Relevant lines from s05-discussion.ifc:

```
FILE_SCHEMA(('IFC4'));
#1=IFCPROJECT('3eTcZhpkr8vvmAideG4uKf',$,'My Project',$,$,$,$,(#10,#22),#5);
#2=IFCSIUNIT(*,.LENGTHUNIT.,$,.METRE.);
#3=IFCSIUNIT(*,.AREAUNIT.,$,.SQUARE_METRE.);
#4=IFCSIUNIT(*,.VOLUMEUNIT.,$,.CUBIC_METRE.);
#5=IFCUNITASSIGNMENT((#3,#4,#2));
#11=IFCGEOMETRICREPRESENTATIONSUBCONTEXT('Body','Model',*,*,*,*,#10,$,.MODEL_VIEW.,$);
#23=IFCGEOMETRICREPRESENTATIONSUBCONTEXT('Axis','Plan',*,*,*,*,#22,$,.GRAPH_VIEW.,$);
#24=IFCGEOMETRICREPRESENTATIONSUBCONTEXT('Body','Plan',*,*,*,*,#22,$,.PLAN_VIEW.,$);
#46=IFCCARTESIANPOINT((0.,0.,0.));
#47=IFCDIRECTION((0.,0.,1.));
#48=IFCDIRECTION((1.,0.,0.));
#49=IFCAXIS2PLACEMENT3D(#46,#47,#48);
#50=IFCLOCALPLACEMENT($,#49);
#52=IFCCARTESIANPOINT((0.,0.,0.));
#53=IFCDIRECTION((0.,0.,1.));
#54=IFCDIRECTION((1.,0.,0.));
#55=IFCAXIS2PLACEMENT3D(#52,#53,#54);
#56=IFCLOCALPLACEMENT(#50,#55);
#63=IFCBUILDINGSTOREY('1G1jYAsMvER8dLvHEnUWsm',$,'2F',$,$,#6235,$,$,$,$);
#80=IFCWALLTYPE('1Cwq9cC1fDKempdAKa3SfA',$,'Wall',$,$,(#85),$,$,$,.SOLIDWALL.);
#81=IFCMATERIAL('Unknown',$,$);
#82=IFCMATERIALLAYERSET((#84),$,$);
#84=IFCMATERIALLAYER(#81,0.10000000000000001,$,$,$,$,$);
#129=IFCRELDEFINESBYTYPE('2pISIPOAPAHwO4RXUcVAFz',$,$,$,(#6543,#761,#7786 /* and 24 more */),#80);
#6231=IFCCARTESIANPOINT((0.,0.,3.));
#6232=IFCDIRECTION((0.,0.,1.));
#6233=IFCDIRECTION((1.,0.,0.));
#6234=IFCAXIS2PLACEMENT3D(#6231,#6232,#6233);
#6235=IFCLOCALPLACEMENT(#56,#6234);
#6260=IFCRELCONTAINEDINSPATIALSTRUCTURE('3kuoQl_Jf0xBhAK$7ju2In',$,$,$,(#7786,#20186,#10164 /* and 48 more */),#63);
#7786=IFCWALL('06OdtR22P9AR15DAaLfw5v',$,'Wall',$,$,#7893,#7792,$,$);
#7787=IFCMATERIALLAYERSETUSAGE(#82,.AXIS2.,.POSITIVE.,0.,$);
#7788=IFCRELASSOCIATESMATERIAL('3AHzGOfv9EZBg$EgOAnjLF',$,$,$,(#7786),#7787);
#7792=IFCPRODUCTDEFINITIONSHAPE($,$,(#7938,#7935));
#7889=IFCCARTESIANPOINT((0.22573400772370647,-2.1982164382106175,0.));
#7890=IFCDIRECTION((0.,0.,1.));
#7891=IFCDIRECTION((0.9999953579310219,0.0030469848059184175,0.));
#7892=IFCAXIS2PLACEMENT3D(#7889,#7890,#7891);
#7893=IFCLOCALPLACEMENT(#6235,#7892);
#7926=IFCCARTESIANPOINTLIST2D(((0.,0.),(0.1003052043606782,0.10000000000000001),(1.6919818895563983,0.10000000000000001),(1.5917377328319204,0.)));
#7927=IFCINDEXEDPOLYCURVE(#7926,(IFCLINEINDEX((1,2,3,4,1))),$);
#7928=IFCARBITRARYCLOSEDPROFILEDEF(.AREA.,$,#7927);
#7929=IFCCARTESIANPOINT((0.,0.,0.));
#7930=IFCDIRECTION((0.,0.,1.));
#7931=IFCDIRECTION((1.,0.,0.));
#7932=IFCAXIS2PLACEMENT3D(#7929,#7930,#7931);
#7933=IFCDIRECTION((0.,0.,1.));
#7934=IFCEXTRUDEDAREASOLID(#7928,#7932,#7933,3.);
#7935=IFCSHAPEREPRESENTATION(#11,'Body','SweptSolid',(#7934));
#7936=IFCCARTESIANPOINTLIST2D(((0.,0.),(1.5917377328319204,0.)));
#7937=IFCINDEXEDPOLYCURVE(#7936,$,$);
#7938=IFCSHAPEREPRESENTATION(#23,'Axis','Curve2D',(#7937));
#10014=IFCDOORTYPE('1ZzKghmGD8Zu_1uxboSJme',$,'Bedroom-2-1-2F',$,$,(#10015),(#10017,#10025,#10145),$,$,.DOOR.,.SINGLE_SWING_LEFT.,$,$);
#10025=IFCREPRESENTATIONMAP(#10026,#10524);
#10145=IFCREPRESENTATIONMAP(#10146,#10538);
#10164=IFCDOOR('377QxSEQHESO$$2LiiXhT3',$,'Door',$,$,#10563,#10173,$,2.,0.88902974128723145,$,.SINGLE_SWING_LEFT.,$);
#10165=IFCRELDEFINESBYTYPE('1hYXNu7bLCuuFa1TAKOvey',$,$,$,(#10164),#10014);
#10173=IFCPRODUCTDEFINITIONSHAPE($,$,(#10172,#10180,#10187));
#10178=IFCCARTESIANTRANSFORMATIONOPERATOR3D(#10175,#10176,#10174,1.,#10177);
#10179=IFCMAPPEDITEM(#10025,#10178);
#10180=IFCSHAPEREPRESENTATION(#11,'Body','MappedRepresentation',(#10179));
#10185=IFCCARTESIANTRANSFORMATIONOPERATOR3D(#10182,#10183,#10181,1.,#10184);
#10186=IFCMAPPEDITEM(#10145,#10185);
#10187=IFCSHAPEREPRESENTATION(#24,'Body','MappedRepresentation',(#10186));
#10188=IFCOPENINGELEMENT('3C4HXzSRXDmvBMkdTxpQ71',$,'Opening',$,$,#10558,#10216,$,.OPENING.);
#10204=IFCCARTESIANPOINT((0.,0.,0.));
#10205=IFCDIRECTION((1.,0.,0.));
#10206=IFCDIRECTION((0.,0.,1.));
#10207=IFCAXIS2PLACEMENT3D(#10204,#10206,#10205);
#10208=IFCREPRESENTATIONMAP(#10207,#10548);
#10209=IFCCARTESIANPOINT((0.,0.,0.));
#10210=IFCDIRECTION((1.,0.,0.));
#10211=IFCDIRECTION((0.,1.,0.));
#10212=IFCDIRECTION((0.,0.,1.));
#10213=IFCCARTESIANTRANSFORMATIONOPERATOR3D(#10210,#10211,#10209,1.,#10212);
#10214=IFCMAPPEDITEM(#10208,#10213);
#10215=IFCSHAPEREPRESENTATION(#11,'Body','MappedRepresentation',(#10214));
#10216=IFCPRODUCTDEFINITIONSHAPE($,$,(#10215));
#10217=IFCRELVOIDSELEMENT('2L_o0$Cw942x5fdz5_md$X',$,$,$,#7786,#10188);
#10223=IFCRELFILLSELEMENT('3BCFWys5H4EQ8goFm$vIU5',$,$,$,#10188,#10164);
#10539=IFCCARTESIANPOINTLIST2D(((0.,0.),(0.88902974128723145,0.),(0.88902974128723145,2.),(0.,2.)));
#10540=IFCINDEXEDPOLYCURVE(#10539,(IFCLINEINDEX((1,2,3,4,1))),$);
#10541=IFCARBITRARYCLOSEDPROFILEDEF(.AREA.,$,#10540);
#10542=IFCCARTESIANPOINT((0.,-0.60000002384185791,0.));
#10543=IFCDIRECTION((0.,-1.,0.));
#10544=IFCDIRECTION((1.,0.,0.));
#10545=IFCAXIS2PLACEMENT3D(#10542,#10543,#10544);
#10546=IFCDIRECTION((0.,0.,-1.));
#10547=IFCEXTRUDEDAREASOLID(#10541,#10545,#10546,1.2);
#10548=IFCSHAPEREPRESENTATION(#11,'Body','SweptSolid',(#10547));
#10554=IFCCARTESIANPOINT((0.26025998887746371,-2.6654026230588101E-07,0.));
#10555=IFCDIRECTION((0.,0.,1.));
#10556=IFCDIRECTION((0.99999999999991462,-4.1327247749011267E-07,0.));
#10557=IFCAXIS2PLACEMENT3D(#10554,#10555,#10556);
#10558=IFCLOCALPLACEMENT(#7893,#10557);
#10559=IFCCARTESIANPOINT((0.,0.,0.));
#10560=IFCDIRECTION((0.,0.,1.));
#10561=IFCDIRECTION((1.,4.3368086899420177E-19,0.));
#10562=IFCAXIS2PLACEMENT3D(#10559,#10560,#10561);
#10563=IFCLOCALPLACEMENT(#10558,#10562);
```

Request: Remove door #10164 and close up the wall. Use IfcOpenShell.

```python
import ifcopenshell
import ifcopenshell.api.feature
import ifcopenshell.api.root
import ifcopenshell.geom
import ifcopenshell.util.shape

model = ifcopenshell.open("s05-discussion.ifc")
settings = ifcopenshell.geom.settings()


def volume(element):
    """Net volume in cubic metres, openings subtracted."""
    shape = ifcopenshell.geom.create_shape(settings, element)
    return ifcopenshell.util.shape.get_volume(shape.geometry)


door = model.by_guid("377QxSEQHESO$$2LiiXhT3")
opening = door.FillsVoids[0].RelatingOpeningElement
wall = opening.VoidsElements[0].RelatingBuildingElement
before = volume(wall)

ifcopenshell.api.root.remove_product(model, product=door)
ifcopenshell.api.feature.remove_feature(model, feature=opening)

after = volume(wall)

print(f"wall volume {before:.3f} -> {after:.3f} m3")

model.write("s05-discussion-out.ifc")
```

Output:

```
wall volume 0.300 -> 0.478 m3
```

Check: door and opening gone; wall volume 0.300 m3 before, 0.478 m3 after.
